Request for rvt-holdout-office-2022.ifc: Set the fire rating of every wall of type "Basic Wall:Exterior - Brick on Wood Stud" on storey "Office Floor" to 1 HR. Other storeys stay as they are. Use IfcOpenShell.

First a look at what the model holds.

```python
import ifcopenshell
import ifcopenshell.util.element

model = ifcopenshell.open("rvt-holdout-office-2022.ifc")
print(model.schema)
storey = next(s for s in model.by_type("IfcBuildingStorey") if s.Name == "Office Floor")
walls = [e for e in ifcopenshell.util.element.get_decomposition(storey) if e.is_a("IfcWall")]
seen = {}
for e in walls:
    element_type = ifcopenshell.util.element.get_type(e)
    key = (element_type.Name if element_type != e and element_type else None, ifcopenshell.util.element.get_pset(e, "Pset_WallCommon", "FireRating"))
    seen[key] = seen.get(key, 0) + 1
for (name, value), count in sorted(seen.items(), key=str):
    print(count, "x", name, "|", value)
```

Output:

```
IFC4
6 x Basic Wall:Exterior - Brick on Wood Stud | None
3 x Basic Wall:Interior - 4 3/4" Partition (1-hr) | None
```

```python
import ifcopenshell
import ifcopenshell.api.pset
import ifcopenshell.util.element

model = ifcopenshell.open("rvt-holdout-office-2022.ifc")

storey = next(s for s in model.by_type("IfcBuildingStorey") if s.Name == "Office Floor")
walls = [e for e in ifcopenshell.util.element.get_decomposition(storey) if e.is_a("IfcWall")]

count = 0
for e in walls:
    element_type = ifcopenshell.util.element.get_type(e)
    if element_type in (None, e) or element_type.Name != "Basic Wall:Exterior - Brick on Wood Stud":
        continue
    # add_pset returns the element's existing set when there is one.
    pset = ifcopenshell.api.pset.add_pset(model, product=e, name="Pset_WallCommon")
    ifcopenshell.api.pset.edit_pset(model, pset=pset, properties={"FireRating": "1 HR"})
    count += 1

print(count, "walls updated")

model.write("rvt-holdout-office-2022_edited.ifc")
```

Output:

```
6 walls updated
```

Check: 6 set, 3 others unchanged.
